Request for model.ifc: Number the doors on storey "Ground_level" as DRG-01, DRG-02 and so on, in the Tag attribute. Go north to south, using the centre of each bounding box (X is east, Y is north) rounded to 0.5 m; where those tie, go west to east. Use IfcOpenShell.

First a look at what the model holds.

```python
import ifcopenshell
import ifcopenshell.util.element
import ifcopenshell.util.placement

model = ifcopenshell.open("model.ifc")
print(model.schema)
storey = next(s for s in model.by_type("IfcBuildingStorey") if s.Name == "Ground_level")
doors = [e for e in ifcopenshell.util.element.get_decomposition(storey) if e.is_a("IfcDoor")]
for e in sorted(doors, key=lambda e: e.id()):
    origin = ifcopenshell.util.placement.get_local_placement(e.ObjectPlacement)[:3, 3]
    print(e.id(), e.Tag, e.Name, origin.round(2) + 0.0, sep=" | ")
```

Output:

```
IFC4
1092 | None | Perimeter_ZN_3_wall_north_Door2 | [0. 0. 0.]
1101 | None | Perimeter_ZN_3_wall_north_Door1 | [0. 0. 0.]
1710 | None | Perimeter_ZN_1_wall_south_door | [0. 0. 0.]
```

```python
import ifcopenshell
import ifcopenshell.geom
import ifcopenshell.util.element
import ifcopenshell.util.shape

model = ifcopenshell.open("model.ifc")
settings = ifcopenshell.geom.settings()
settings.set("use-world-coords", True)


def centre(element):
    shape = ifcopenshell.geom.create_shape(settings, element)
    return ifcopenshell.util.shape.get_bbox_centroid(shape.geometry)


storey = next(s for s in model.by_type("IfcBuildingStorey") if s.Name == "Ground_level")
doors = [e for e in ifcopenshell.util.element.get_decomposition(storey) if e.is_a("IfcDoor")]

# Insertion points can sit at a corner or the storey origin, so sort by the geometry (in metres).
centres = {e: centre(e) for e in doors}
doors.sort(key=lambda e: (-round(centres[e][1] / 0.5), centres[e][0]))

for i, e in enumerate(doors, start=1):
    number = f"DRG-{i:02d}"
    e.Tag = number
    print(e.id(), number)

model.write("model_updated.ifc")
```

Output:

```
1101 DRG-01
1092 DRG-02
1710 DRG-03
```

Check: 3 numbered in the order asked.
